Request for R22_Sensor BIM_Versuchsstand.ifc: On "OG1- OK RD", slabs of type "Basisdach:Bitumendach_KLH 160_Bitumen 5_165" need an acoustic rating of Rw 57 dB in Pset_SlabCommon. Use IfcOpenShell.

First a look at what the model holds.

```python
import ifcopenshell
import ifcopenshell.util.element

model = ifcopenshell.open("R22_Sensor BIM_Versuchsstand.ifc")
print(model.schema)
storey = next(s for s in model.by_type("IfcBuildingStorey") if s.Name == "OG1- OK RD")
slabs = [e for e in ifcopenshell.util.element.get_decomposition(storey) if e.is_a("IfcSlab")]
seen = {}
for e in slabs:
    element_type = ifcopenshell.util.element.get_type(e)
    key = (element_type.Name if element_type != e and element_type else None, ifcopenshell.util.element.get_pset(e, "Pset_SlabCommon", "AcousticRating"))
    seen[key] = seen.get(key, 0) + 1
for (name, value), count in sorted(seen.items(), key=str):
    print(count, "x", name, "|", value)
```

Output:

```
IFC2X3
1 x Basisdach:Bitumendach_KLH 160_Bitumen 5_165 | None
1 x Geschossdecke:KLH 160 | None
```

```python
import ifcopenshell
import ifcopenshell.api.pset
import ifcopenshell.util.element

model = ifcopenshell.open("R22_Sensor BIM_Versuchsstand.ifc")

storey = next(s for s in model.by_type("IfcBuildingStorey") if s.Name == "OG1- OK RD")
slabs = [e for e in ifcopenshell.util.element.get_decomposition(storey) if e.is_a("IfcSlab")]

count = 0
for e in slabs:
    element_type = ifcopenshell.util.element.get_type(e)
    if element_type in (None, e) or element_type.Name != "Basisdach:Bitumendach_KLH 160_Bitumen 5_165":
        continue
    # add_pset returns the element's existing set when there is one.
    pset = ifcopenshell.api.pset.add_pset(model, product=e, name="Pset_SlabCommon")
    ifcopenshell.api.pset.edit_pset(model, pset=pset, properties={"AcousticRating": "Rw 57 dB"})
    count += 1

print(count, "slabs updated")

model.write("R22_Sensor BIM_Versuchsstand_rev.ifc")
```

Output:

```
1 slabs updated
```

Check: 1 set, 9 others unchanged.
